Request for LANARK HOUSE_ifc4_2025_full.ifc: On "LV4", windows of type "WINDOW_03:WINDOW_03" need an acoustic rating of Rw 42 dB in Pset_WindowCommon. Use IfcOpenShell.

First a look at what the model holds.

```python
import ifcopenshell
import ifcopenshell.util.element

model = ifcopenshell.open("LANARK HOUSE_ifc4_2025_full.ifc")
print(model.schema)
storey = next(s for s in model.by_type("IfcBuildingStorey") if s.Name == "LV4")
windows = [e for e in ifcopenshell.util.element.get_decomposition(storey) if e.is_a("IfcWindow")]
seen = {}
for e in windows:
    element_type = ifcopenshell.util.element.get_type(e)
    key = (element_type.Name if element_type != e and element_type else None, ifcopenshell.util.element.get_pset(e, "Pset_WindowCommon", "AcousticRating"))
    seen[key] = seen.get(key, 0) + 1
for (name, value), count in sorted(seen.items(), key=str):
    print(count, "x", name, "|", value)
```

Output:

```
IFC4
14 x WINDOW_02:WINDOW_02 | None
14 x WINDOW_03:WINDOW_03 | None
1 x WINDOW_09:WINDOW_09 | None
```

```python
import ifcopenshell
import ifcopenshell.api.pset
import ifcopenshell.util.element

model = ifcopenshell.open("LANARK HOUSE_ifc4_2025_full.ifc")

storey = next(s for s in model.by_type("IfcBuildingStorey") if s.Name == "LV4")
windows = [e for e in ifcopenshell.util.element.get_decomposition(storey) if e.is_a("IfcWindow")]

count = 0
for e in windows:
    element_type = ifcopenshell.util.element.get_type(e)
    if element_type in (None, e) or element_type.Name != "WINDOW_03:WINDOW_03":
        continue
    # add_pset returns the element's existing set when there is one.
    pset = ifcopenshell.api.pset.add_pset(model, product=e, name="Pset_WindowCommon")
    ifcopenshell.api.pset.edit_pset(model, pset=pset, properties={"AcousticRating": "Rw 42 dB"})
    count += 1

print(count, "windows updated")

model.write("LANARK HOUSE_ifc4_2025_full_updated.ifc")
```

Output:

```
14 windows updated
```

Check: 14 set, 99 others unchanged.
